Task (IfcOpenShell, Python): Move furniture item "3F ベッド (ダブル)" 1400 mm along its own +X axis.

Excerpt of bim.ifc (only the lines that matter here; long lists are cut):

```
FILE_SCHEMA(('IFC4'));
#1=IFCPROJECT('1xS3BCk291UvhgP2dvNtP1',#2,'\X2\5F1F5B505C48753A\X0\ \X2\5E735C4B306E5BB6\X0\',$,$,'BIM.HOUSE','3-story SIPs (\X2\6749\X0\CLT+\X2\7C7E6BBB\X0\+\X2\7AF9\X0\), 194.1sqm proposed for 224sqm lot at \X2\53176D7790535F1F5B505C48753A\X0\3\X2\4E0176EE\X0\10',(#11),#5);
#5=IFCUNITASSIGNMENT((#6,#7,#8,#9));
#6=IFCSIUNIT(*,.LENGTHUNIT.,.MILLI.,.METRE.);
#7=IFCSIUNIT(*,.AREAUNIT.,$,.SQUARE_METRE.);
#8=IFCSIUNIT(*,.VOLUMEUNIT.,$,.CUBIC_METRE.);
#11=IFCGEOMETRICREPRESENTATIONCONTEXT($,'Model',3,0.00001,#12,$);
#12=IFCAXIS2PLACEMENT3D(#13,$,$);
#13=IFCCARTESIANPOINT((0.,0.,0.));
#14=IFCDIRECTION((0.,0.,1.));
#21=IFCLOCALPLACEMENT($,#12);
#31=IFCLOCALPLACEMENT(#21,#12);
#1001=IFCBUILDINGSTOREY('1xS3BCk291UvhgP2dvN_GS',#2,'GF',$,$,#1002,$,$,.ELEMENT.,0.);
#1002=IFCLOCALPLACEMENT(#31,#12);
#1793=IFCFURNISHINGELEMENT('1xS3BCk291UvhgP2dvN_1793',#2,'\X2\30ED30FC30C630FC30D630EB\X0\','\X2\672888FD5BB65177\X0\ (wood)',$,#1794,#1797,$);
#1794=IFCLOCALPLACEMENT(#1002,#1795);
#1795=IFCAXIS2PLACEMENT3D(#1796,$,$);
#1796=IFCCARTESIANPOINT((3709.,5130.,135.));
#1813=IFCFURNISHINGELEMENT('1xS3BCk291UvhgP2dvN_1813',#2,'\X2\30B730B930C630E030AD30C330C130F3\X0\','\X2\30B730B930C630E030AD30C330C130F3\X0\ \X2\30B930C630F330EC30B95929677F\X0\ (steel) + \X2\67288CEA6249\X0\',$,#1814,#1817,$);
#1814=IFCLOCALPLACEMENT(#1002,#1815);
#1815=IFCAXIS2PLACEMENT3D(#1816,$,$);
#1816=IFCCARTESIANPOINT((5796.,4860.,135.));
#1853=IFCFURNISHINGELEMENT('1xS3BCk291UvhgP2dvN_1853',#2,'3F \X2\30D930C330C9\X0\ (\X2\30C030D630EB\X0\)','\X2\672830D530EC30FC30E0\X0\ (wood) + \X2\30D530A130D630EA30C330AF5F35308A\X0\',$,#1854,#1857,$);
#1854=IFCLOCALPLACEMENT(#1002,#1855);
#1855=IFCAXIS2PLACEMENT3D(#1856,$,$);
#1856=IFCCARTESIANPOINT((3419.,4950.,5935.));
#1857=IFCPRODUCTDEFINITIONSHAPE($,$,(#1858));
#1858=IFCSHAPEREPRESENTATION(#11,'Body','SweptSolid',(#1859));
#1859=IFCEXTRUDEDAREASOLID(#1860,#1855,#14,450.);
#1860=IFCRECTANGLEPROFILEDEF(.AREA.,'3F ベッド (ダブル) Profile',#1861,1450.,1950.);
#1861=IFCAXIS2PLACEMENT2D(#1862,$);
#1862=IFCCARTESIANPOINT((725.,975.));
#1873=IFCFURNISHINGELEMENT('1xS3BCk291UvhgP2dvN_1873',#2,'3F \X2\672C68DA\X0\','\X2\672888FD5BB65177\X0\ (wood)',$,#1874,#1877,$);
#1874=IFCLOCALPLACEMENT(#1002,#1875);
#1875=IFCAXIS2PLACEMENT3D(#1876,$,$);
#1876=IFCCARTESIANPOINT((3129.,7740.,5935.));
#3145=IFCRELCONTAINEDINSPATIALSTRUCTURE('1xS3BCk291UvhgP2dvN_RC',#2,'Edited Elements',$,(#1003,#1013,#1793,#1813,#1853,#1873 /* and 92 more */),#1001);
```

```python
import ifcopenshell
import ifcopenshell.api.geometry
import ifcopenshell.util.placement
import ifcopenshell.util.unit

model = ifcopenshell.open("bim.ifc")
unit_scale = ifcopenshell.util.unit.calculate_unit_scale(model)

item = model.by_guid("1xS3BCk291UvhgP2dvN_1853")
matrix = ifcopenshell.util.placement.get_local_placement(item.ObjectPlacement)
matrix[:3, 3] += matrix[:3, 0] * 1.4 / unit_scale
ifcopenshell.api.geometry.edit_object_placement(model, product=item, matrix=matrix, is_si=False)

print(ifcopenshell.util.placement.get_local_placement(item.ObjectPlacement).round(3) + 0.0)

model.write("bim_updated.ifc")
```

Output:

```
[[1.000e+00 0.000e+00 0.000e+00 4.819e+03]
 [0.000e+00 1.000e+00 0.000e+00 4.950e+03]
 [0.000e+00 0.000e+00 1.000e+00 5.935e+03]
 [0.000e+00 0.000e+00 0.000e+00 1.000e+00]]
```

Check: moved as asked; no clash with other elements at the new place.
